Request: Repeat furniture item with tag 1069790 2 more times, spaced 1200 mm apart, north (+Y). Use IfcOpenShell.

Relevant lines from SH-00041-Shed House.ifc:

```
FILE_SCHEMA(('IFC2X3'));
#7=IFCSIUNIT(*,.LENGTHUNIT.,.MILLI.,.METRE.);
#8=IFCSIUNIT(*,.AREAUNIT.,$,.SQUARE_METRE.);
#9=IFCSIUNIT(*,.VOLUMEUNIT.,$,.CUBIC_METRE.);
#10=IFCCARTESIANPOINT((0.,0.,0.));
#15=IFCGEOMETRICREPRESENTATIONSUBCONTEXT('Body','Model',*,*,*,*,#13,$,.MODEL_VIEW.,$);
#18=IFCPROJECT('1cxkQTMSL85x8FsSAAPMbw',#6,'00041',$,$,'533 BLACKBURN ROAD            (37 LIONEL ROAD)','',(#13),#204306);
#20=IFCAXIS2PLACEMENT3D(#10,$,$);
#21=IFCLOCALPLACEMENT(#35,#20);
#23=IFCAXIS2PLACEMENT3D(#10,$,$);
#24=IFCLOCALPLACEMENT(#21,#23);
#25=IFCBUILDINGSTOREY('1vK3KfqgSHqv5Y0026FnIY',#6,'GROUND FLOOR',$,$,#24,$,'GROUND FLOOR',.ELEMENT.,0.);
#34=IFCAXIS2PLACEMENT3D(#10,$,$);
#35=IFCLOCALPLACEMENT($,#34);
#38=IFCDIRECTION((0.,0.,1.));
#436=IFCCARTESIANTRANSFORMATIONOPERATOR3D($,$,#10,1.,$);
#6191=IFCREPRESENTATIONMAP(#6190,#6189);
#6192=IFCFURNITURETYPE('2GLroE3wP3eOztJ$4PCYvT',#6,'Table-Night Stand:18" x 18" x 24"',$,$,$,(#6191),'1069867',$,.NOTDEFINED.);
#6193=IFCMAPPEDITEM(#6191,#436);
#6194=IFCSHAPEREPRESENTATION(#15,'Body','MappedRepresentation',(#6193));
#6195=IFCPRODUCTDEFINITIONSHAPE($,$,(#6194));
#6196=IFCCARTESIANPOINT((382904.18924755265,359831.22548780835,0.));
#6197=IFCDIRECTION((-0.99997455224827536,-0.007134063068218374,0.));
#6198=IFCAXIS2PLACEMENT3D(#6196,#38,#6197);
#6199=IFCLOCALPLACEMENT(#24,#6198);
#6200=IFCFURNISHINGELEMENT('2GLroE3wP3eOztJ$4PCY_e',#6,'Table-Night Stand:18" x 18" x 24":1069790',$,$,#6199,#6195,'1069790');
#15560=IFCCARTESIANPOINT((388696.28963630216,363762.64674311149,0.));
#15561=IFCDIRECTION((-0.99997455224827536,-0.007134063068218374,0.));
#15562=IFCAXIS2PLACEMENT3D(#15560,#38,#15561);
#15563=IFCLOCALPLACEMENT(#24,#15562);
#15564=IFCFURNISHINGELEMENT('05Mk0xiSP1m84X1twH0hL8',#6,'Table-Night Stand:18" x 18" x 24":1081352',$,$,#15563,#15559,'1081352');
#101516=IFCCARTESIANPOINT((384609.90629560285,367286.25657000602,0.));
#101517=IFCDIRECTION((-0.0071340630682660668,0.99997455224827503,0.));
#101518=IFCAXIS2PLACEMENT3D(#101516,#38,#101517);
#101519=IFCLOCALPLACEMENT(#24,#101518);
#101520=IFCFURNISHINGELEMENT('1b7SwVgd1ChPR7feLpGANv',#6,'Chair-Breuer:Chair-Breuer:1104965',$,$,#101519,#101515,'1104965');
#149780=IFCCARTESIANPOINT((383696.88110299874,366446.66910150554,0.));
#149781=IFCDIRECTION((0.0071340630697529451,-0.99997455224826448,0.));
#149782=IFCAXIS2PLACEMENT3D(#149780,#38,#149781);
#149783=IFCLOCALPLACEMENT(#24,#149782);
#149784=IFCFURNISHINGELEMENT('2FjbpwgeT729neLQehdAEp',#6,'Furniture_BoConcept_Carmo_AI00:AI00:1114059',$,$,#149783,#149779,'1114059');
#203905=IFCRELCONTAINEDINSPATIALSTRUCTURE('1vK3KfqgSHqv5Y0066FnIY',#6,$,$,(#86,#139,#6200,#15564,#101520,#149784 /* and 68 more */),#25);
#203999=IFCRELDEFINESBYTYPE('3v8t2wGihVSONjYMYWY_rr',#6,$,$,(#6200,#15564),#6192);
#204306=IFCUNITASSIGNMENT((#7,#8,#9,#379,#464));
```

```python
import numpy as np
import ifcopenshell
import ifcopenshell.api.geometry
import ifcopenshell.api.root
import ifcopenshell.util.element
import ifcopenshell.util.placement

model = ifcopenshell.open("SH-00041-Shed House.ifc")


def reuse_history(source, copy):
    """copy_class also copies each property set's owner history, people and application; keep the originals."""
    for rel in copy.IsDefinedBy:
        if rel.is_a("IfcRelDefinesByProperties") and (history := rel.RelatingPropertyDefinition.OwnerHistory):
            rel.RelatingPropertyDefinition.OwnerHistory = source.OwnerHistory
            ifcopenshell.util.element.remove_deep2(model, history)


source = model.by_id(6200)
base = ifcopenshell.util.placement.get_local_placement(source.ObjectPlacement)
step = np.array([0.0, 1.0, 0.0]) * 1200.0

for i in range(1, 3):
    copy = ifcopenshell.api.root.copy_class(model, product=source)
    copy.Representation = ifcopenshell.util.element.copy_deep(
        model, source.Representation, exclude=["IfcGeometricRepresentationContext", "IfcRepresentationMap"]
    )
    copy.Name = 'Table-Night Stand:18" x 18" x 24"'
    copy.Tag = None
    reuse_history(source, copy)
    matrix = base.copy()
    matrix[:3, 3] += i * step
    print("added at", matrix[:3, 3].round(3) + 0.0)
    ifcopenshell.api.geometry.edit_object_placement(model, product=copy, matrix=matrix, is_si=False)

model.write("SH-00041-Shed House_rev.ifc")
```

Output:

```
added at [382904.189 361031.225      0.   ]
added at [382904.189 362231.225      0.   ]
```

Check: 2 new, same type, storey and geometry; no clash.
